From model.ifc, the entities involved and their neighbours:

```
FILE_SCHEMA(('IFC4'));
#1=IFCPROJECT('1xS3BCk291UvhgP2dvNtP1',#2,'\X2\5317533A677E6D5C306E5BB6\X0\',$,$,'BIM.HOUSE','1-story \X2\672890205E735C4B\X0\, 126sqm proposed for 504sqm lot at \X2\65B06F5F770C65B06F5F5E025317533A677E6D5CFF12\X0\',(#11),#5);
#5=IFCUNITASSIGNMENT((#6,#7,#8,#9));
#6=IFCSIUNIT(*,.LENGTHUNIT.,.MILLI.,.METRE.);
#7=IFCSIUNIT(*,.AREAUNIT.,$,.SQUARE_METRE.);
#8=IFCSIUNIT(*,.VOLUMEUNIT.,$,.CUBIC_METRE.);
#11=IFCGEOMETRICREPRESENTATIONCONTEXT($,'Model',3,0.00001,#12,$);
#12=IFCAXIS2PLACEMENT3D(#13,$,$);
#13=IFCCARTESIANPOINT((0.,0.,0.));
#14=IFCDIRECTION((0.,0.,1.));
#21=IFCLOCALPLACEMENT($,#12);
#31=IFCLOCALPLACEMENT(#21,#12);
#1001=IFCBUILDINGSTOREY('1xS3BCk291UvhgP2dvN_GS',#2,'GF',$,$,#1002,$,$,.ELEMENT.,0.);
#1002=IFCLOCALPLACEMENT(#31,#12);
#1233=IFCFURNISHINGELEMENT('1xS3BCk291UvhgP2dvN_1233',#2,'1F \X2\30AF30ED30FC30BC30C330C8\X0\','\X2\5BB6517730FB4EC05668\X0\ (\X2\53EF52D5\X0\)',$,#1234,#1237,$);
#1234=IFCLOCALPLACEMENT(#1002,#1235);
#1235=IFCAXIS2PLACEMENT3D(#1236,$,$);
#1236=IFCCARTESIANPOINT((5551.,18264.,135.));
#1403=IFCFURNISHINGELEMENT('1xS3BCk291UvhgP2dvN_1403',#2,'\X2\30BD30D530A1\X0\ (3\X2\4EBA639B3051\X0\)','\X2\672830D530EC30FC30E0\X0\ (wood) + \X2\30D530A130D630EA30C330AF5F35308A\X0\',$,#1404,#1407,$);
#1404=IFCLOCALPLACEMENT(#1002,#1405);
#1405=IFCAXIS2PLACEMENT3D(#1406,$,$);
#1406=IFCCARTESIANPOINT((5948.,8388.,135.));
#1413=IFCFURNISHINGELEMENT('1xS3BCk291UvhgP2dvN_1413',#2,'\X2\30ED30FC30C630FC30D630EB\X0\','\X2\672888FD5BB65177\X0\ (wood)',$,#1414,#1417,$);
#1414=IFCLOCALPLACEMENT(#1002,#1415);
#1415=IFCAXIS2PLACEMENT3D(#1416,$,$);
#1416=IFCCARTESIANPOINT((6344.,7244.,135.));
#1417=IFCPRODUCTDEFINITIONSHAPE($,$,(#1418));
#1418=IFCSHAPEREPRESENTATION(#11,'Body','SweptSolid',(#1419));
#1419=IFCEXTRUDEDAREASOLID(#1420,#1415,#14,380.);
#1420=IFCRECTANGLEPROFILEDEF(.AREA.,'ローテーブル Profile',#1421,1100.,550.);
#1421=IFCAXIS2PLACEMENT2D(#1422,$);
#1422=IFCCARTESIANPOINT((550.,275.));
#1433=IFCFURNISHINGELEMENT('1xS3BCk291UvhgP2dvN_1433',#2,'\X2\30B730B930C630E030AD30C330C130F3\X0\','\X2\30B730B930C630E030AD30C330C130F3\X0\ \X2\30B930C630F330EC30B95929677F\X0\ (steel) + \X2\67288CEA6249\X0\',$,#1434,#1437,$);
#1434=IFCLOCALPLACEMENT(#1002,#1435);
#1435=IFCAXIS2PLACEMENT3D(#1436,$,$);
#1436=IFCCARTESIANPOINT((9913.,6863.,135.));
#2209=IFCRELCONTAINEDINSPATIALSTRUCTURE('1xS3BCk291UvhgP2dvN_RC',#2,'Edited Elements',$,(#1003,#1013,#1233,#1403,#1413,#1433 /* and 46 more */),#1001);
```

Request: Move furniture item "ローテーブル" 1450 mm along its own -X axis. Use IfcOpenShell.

```python
import ifcopenshell
import ifcopenshell.api.geometry
import ifcopenshell.util.placement
import ifcopenshell.util.unit

model = ifcopenshell.open("model.ifc")
unit_scale = ifcopenshell.util.unit.calculate_unit_scale(model)

item = model.by_guid("1xS3BCk291UvhgP2dvN_1413")
matrix = ifcopenshell.util.placement.get_local_placement(item.ObjectPlacement)
matrix[:3, 3] -= matrix[:3, 0] * 1.45 / unit_scale
ifcopenshell.api.geometry.edit_object_placement(model, product=item, matrix=matrix, is_si=False)

print(ifcopenshell.util.placement.get_local_placement(item.ObjectPlacement).round(3) + 0.0)

model.write("model_v2.ifc")
```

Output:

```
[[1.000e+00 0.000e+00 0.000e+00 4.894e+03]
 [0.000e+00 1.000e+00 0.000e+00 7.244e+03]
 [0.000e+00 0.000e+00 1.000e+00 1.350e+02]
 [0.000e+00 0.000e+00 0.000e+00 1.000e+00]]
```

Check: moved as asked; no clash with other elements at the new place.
